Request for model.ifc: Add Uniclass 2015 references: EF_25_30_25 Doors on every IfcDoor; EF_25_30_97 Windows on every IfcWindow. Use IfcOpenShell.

First a look at what the model holds.

```python
import ifcopenshell

model = ifcopenshell.open("model.ifc")
print(model.schema)
print("classifications:", [c.Name for c in model.by_type("IfcClassification")])
for ifc_class in ("IfcDoor", "IfcRoof", "IfcStair", "IfcWall", "IfcWindow"):
    print(ifc_class, len(model.by_type(ifc_class)))
```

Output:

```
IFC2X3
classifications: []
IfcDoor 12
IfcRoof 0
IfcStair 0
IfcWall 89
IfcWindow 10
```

```python
import ifcopenshell
import ifcopenshell.api.classification

model = ifcopenshell.open("model.ifc")

# IFC2X3 requires Source and Edition and has no link from the project to the system.
system = model.create_entity("IfcClassification", Source="NBS", Edition="2015", Name="Uniclass 2015")

codes = {
    "IfcDoor": ("EF_25_30_25", "Doors"),
    "IfcWindow": ("EF_25_30_97", "Windows"),
}
for ifc_class, (code, name) in codes.items():
    products = model.by_type(ifc_class)
    ifcopenshell.api.classification.add_reference(
        model, products=products, classification=system, identification=code, name=name
    )
    print(code, len(products))

model.write("model_edited.ifc")
```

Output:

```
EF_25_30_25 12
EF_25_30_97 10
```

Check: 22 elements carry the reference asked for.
